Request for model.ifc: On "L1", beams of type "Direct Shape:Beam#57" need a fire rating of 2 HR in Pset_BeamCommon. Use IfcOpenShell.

First a look at what the model holds.

```python
import ifcopenshell
import ifcopenshell.util.element

model = ifcopenshell.open("model.ifc")
print(model.schema)
storey = next(s for s in model.by_type("IfcBuildingStorey") if s.Name == "L1")
beams = [e for e in ifcopenshell.util.element.get_decomposition(storey) if e.is_a("IfcBeam")]
seen = {}
for e in beams:
    element_type = ifcopenshell.util.element.get_type(e)
    key = (element_type.Name if element_type != e and element_type else None, ifcopenshell.util.element.get_pset(e, "Pset_BeamCommon", "FireRating"))
    seen[key] = seen.get(key, 0) + 1
for (name, value), count in sorted(seen.items(), key=str):
    print(count, "x", name, "|", value)
```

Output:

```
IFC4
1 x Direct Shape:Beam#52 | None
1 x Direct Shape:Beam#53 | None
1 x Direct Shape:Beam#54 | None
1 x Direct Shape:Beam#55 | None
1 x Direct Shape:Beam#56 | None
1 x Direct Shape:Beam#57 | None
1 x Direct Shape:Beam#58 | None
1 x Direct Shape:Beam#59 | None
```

```python
import ifcopenshell
import ifcopenshell.api.pset
import ifcopenshell.util.element

model = ifcopenshell.open("model.ifc")

storey = next(s for s in model.by_type("IfcBuildingStorey") if s.Name == "L1")
beams = [e for e in ifcopenshell.util.element.get_decomposition(storey) if e.is_a("IfcBeam")]

count = 0
for e in beams:
    element_type = ifcopenshell.util.element.get_type(e)
    if element_type in (None, e) or element_type.Name != "Direct Shape:Beam#57":
        continue
    # add_pset returns the element's existing set when there is one.
    pset = ifcopenshell.api.pset.add_pset(model, product=e, name="Pset_BeamCommon")
    ifcopenshell.api.pset.edit_pset(model, pset=pset, properties={"FireRating": "2 HR"})
    count += 1

print(count, "beams updated")

model.write("model_updated.ifc")
```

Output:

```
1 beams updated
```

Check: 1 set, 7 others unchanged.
